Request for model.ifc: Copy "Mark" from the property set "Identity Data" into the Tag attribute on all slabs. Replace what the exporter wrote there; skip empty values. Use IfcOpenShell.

First a look at what the model holds.

```python
import ifcopenshell
import ifcopenshell.util.element

model = ifcopenshell.open("model.ifc")
print(model.schema)
slabs = model.by_type("IfcSlab")
print(len(slabs), "slabs")
for e in slabs[:8]:
    source = ifcopenshell.util.element.get_pset(e, "Identity Data", "Mark")
    target = e.Tag
    print(e.id(), repr(source), repr(target), sep=" | ")
```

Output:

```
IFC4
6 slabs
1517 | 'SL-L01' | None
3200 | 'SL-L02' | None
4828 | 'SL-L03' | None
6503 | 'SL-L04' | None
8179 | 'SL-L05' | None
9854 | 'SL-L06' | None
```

```python
import ifcopenshell
import ifcopenshell.util.element

model = ifcopenshell.open("model.ifc")

count = 0
for e in model.by_type("IfcSlab"):
    value = ifcopenshell.util.element.get_pset(e, "Identity Data", "Mark")
    current = e.Tag
    if not value or not value.strip() or current == value:
        continue
    e.Tag = value
    count += 1

print(count, "slabs updated")

model.write("model_edited.ifc")
```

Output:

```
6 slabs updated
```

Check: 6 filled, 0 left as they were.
